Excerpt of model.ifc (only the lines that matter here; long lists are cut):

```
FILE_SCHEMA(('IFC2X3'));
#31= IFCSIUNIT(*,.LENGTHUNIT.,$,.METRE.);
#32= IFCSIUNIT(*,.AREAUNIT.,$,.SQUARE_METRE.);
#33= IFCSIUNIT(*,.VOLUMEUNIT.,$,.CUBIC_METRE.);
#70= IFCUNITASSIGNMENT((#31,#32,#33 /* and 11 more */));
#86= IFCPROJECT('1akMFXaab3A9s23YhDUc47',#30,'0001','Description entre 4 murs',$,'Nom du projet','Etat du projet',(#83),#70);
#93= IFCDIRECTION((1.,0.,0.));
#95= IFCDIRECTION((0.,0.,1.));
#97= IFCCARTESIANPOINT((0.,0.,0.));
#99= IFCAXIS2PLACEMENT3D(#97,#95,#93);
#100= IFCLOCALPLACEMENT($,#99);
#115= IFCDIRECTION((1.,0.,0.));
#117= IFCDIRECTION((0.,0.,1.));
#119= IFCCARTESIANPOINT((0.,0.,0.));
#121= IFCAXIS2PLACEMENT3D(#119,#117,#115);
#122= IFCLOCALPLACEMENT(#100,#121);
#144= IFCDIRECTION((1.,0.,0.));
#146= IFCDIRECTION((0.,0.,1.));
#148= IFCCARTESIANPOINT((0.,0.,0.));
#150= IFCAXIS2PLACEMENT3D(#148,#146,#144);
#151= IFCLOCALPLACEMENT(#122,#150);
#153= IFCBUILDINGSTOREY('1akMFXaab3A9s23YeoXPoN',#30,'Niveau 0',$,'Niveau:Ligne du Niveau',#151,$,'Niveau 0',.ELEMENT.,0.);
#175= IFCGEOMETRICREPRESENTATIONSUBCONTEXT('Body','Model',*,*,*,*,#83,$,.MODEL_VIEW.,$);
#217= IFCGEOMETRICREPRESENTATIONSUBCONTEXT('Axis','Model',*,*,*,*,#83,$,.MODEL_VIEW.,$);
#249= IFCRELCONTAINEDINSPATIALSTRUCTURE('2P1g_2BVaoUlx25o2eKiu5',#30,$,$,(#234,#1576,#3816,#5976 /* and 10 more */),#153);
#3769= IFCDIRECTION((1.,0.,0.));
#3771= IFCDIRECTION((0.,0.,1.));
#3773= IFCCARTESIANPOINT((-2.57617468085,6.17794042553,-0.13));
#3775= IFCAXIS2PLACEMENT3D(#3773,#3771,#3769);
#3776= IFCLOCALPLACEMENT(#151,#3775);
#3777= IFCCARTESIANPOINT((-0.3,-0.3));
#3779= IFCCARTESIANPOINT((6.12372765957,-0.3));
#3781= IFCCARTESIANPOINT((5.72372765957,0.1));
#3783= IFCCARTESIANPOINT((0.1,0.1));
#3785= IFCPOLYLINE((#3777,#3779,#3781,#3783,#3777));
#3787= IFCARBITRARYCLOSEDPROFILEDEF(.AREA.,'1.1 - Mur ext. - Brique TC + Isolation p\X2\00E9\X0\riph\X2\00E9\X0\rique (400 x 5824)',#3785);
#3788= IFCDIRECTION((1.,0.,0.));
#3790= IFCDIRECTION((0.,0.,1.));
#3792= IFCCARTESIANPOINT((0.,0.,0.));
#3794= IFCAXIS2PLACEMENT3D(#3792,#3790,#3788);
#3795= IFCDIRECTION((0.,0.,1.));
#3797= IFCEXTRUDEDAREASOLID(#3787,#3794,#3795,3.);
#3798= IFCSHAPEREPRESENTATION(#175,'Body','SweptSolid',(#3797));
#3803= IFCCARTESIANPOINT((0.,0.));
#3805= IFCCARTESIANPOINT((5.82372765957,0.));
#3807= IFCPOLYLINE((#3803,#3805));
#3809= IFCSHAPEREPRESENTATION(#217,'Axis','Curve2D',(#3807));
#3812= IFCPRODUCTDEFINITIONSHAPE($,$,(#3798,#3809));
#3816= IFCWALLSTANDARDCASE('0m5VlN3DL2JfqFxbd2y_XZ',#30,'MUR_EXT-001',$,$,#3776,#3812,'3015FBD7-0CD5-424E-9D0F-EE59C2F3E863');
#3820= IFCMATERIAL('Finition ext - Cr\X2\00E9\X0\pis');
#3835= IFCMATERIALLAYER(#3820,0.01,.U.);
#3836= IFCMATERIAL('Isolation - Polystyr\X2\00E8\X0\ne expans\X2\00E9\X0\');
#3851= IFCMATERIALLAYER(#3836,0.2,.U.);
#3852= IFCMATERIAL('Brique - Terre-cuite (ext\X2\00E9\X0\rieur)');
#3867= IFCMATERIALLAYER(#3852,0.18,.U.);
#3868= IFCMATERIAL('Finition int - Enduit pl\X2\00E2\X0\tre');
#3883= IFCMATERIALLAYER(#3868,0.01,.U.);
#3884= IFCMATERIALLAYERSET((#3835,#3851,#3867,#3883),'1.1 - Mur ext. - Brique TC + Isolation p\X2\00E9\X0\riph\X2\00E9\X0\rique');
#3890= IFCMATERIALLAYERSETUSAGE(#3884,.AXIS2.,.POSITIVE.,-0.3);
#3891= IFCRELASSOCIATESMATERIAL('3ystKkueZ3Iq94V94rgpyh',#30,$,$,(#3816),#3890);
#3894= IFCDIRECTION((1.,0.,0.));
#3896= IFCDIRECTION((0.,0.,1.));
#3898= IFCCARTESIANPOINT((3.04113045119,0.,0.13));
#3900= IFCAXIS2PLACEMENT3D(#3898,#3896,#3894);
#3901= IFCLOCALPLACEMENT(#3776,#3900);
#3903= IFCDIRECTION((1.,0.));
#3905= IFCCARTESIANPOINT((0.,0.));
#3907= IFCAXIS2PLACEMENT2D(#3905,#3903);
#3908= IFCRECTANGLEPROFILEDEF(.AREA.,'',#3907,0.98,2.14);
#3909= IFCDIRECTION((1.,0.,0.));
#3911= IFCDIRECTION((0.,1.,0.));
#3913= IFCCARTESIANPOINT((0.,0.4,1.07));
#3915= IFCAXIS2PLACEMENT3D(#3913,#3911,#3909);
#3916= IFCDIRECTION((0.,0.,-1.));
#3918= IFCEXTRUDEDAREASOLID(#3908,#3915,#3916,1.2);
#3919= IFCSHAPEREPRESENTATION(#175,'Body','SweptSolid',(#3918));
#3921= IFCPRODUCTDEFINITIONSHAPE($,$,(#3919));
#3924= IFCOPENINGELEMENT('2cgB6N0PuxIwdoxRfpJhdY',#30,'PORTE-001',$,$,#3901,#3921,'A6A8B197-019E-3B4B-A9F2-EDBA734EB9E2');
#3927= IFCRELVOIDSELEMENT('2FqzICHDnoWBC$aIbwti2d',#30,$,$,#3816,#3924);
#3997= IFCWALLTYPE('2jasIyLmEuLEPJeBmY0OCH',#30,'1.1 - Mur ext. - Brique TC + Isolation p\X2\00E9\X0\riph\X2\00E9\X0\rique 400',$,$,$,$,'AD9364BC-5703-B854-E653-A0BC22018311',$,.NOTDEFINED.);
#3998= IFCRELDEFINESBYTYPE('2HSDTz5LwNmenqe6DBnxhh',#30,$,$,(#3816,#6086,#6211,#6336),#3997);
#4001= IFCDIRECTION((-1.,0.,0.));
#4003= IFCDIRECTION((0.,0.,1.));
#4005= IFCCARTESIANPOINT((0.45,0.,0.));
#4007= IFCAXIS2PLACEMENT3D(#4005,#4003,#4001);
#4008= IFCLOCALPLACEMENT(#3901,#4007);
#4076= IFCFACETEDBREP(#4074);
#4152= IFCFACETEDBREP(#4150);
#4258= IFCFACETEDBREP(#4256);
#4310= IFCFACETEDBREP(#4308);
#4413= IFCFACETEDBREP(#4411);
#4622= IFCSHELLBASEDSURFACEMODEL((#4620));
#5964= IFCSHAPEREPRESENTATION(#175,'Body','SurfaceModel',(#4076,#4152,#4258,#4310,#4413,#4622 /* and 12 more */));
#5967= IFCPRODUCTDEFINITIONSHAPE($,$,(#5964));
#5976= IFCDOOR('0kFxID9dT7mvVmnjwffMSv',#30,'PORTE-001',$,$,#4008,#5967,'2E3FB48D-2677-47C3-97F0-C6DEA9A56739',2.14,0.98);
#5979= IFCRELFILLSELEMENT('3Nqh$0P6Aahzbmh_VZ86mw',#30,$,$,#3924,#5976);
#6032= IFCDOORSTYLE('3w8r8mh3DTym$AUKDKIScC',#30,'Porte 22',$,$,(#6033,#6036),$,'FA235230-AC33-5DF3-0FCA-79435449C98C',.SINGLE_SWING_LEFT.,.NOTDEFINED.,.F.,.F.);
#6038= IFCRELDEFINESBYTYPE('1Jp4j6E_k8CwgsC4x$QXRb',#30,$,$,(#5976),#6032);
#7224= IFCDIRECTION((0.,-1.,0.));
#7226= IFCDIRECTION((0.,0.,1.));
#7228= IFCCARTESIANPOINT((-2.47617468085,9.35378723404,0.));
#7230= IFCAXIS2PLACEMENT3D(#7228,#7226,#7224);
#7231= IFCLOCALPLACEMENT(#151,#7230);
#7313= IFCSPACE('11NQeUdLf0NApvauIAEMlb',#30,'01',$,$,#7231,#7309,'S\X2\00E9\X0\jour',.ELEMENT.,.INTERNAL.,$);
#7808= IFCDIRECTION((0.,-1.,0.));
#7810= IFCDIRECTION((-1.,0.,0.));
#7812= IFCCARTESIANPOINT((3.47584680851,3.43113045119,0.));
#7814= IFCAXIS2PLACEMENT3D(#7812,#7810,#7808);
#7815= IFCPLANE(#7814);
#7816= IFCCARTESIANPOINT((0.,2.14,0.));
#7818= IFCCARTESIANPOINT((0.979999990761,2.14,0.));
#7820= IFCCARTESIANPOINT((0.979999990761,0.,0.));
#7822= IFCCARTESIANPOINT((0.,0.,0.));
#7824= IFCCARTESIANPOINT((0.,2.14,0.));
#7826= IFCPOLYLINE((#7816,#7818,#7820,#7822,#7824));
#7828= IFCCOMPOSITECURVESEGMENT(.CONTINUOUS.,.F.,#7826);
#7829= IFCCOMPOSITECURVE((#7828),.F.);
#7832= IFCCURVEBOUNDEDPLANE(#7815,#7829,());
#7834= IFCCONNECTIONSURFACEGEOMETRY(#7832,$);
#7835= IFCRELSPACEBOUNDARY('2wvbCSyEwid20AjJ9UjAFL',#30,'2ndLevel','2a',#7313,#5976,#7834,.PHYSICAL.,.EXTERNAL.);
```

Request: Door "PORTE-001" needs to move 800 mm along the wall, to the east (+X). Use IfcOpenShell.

```python
import numpy as np
import ifcopenshell
import ifcopenshell.api.geometry
import ifcopenshell.util.placement
import ifcopenshell.util.unit

model = ifcopenshell.open("model.ifc")
unit_scale = ifcopenshell.util.unit.calculate_unit_scale(model)

door = model.by_id(5976)
opening = door.FillsVoids[0].RelatingOpeningElement
wall = opening.VoidsElements[0].RelatingBuildingElement

wall_matrix = ifcopenshell.util.placement.get_local_placement(wall.ObjectPlacement)
shift = wall_matrix[:3, 0] * 0.8 / unit_scale
before = ifcopenshell.util.placement.get_local_placement(door.ObjectPlacement)[:3, 3].copy()

# The door is placed relative to its opening, so it follows when the opening moves.
matrix = ifcopenshell.util.placement.get_local_placement(opening.ObjectPlacement)
matrix[:3, 3] += shift
ifcopenshell.api.geometry.edit_object_placement(
    model, product=opening, matrix=matrix, is_si=False, should_transform_children=True
)

# Space boundary surfaces are stored in each space's coordinates; move them too.
for rel in door.ProvidesBoundaries:
    if not rel.ConnectionGeometry:
        continue
    surface = rel.ConnectionGeometry.SurfaceOnRelatingElement.BasisSurface
    space_matrix = ifcopenshell.util.placement.get_local_placement(rel.RelatingSpace.ObjectPlacement)
    point = np.array(surface.Position.Location.Coordinates) + space_matrix[:3, :3].T @ shift
    surface.Position = model.createIfcAxis2Placement3D(
        model.createIfcCartesianPoint(point.tolist()), surface.Position.Axis, surface.Position.RefDirection
    )

after = ifcopenshell.util.placement.get_local_placement(door.ObjectPlacement)[:3, 3]
print("door moved by", (after - before).round(3) + 0.0)

model.write("model_updated.ifc")
```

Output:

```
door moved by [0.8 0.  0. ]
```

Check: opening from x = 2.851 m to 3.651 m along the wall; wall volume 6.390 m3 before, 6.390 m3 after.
